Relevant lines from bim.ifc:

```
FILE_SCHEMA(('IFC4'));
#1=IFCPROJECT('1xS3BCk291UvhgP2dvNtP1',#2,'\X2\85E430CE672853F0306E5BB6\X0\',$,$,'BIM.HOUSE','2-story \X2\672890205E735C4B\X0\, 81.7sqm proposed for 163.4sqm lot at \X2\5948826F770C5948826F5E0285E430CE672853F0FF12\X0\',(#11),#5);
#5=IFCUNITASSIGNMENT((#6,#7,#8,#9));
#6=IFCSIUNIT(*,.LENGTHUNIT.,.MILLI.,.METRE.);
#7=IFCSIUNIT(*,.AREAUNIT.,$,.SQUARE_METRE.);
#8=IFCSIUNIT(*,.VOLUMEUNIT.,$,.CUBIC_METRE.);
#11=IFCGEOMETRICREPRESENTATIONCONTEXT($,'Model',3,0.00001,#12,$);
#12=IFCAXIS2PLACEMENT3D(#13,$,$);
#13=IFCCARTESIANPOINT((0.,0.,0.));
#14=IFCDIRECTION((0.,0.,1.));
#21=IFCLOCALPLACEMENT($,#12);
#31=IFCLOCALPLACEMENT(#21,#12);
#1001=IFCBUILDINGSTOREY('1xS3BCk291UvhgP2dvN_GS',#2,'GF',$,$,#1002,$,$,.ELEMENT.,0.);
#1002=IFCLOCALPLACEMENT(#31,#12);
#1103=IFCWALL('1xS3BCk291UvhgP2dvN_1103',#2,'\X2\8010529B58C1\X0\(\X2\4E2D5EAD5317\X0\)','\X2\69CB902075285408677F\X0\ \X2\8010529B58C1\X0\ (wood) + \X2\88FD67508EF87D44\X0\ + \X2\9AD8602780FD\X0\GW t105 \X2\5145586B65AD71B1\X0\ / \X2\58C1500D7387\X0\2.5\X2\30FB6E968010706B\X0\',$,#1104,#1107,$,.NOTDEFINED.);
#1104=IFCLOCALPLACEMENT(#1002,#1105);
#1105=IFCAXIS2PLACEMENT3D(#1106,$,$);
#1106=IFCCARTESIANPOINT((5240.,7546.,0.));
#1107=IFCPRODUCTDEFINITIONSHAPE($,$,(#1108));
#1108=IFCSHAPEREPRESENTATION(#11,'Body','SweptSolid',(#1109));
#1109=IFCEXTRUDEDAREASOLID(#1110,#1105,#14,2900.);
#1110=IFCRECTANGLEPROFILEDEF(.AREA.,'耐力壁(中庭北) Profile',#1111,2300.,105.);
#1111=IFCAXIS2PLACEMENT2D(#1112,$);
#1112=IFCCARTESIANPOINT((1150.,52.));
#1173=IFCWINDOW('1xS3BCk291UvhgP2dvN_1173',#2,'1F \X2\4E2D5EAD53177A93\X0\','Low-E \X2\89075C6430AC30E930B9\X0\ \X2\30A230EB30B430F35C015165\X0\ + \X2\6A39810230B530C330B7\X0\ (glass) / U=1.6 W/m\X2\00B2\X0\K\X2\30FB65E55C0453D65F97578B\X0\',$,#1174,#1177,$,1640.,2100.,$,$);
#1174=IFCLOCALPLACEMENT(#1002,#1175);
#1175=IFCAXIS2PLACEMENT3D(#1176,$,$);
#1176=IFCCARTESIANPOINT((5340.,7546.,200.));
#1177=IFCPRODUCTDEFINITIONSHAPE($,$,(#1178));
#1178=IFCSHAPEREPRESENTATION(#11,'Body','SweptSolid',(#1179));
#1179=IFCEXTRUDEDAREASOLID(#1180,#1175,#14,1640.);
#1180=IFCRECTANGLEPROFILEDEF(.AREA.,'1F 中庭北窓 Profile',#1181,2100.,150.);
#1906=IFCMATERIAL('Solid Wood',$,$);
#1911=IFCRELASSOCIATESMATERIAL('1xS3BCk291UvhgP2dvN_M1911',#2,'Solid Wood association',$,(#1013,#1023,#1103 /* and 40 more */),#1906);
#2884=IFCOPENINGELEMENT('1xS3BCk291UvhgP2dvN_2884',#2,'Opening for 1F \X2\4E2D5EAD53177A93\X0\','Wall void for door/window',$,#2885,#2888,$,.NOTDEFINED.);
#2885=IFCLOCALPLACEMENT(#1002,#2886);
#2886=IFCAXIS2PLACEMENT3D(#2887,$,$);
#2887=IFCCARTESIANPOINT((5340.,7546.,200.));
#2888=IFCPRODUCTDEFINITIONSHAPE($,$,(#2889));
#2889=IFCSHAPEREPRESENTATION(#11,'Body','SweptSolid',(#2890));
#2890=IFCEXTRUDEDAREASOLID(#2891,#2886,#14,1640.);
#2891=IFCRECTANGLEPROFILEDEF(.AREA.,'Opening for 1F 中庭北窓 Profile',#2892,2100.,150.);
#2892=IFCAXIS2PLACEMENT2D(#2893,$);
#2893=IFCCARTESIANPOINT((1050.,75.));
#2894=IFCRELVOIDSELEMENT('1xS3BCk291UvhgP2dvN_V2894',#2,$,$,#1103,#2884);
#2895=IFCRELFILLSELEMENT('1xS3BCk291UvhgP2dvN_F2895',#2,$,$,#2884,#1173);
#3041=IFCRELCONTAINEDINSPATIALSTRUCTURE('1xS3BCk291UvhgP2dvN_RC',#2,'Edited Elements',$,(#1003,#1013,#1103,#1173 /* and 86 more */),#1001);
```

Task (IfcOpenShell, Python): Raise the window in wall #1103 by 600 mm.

```python
import numpy as np
import ifcopenshell
import ifcopenshell.api.geometry
import ifcopenshell.util.placement
import ifcopenshell.util.unit

model = ifcopenshell.open("bim.ifc")
unit_scale = ifcopenshell.util.unit.calculate_unit_scale(model)

window = model.by_guid("1xS3BCk291UvhgP2dvN_1173")
opening = window.FillsVoids[0].RelatingOpeningElement
dz = 600.0

shift = np.array([0.0, 0.0, dz])
# The window is not placed relative to its opening, so move both.
for product in (opening, window):
    matrix = ifcopenshell.util.placement.get_local_placement(product.ObjectPlacement)
    matrix[:3, 3] += shift
    ifcopenshell.api.geometry.edit_object_placement(model, product=product, matrix=matrix, is_si=False)

print(f"moved by {dz * unit_scale:+.3f} m")

model.write("bim_rev.ifc")
```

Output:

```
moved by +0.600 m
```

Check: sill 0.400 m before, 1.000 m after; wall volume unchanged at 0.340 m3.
